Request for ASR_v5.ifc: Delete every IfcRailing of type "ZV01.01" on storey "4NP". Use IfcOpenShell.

First a look at what the model holds.

```python
import ifcopenshell
import ifcopenshell.util.element

model = ifcopenshell.open("ASR_v5.ifc")
print(model.schema)
storey = next(s for s in model.by_type("IfcBuildingStorey") if s.Name == "4NP")
railings = [e for e in ifcopenshell.util.element.get_decomposition(storey) if e.is_a("IfcRailing")]
seen = {}
for e in railings:
    element_type = ifcopenshell.util.element.get_type(e)
    name = element_type.Name if element_type not in (None, e) else None
    seen[name] = seen.get(name, 0) + 1
for name, count in sorted(seen.items(), key=str):
    print(count, "x", name)
```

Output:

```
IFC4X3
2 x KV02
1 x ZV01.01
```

```python
import ifcopenshell
import ifcopenshell.api.root
import ifcopenshell.util.element

model = ifcopenshell.open("ASR_v5.ifc")

storey = next(s for s in model.by_type("IfcBuildingStorey") if s.Name == "4NP")
railings = [e for e in ifcopenshell.util.element.get_decomposition(storey) if e.is_a("IfcRailing")]
targets = [e for e in railings if (t := ifcopenshell.util.element.get_type(e)) not in (None, e) and t.Name == "ZV01.01"]

for e in targets:
    ifcopenshell.api.root.remove_product(model, product=e)
print(len(targets), "removed")

model.write("ASR_v5_edited.ifc")
```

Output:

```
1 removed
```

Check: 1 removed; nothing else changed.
